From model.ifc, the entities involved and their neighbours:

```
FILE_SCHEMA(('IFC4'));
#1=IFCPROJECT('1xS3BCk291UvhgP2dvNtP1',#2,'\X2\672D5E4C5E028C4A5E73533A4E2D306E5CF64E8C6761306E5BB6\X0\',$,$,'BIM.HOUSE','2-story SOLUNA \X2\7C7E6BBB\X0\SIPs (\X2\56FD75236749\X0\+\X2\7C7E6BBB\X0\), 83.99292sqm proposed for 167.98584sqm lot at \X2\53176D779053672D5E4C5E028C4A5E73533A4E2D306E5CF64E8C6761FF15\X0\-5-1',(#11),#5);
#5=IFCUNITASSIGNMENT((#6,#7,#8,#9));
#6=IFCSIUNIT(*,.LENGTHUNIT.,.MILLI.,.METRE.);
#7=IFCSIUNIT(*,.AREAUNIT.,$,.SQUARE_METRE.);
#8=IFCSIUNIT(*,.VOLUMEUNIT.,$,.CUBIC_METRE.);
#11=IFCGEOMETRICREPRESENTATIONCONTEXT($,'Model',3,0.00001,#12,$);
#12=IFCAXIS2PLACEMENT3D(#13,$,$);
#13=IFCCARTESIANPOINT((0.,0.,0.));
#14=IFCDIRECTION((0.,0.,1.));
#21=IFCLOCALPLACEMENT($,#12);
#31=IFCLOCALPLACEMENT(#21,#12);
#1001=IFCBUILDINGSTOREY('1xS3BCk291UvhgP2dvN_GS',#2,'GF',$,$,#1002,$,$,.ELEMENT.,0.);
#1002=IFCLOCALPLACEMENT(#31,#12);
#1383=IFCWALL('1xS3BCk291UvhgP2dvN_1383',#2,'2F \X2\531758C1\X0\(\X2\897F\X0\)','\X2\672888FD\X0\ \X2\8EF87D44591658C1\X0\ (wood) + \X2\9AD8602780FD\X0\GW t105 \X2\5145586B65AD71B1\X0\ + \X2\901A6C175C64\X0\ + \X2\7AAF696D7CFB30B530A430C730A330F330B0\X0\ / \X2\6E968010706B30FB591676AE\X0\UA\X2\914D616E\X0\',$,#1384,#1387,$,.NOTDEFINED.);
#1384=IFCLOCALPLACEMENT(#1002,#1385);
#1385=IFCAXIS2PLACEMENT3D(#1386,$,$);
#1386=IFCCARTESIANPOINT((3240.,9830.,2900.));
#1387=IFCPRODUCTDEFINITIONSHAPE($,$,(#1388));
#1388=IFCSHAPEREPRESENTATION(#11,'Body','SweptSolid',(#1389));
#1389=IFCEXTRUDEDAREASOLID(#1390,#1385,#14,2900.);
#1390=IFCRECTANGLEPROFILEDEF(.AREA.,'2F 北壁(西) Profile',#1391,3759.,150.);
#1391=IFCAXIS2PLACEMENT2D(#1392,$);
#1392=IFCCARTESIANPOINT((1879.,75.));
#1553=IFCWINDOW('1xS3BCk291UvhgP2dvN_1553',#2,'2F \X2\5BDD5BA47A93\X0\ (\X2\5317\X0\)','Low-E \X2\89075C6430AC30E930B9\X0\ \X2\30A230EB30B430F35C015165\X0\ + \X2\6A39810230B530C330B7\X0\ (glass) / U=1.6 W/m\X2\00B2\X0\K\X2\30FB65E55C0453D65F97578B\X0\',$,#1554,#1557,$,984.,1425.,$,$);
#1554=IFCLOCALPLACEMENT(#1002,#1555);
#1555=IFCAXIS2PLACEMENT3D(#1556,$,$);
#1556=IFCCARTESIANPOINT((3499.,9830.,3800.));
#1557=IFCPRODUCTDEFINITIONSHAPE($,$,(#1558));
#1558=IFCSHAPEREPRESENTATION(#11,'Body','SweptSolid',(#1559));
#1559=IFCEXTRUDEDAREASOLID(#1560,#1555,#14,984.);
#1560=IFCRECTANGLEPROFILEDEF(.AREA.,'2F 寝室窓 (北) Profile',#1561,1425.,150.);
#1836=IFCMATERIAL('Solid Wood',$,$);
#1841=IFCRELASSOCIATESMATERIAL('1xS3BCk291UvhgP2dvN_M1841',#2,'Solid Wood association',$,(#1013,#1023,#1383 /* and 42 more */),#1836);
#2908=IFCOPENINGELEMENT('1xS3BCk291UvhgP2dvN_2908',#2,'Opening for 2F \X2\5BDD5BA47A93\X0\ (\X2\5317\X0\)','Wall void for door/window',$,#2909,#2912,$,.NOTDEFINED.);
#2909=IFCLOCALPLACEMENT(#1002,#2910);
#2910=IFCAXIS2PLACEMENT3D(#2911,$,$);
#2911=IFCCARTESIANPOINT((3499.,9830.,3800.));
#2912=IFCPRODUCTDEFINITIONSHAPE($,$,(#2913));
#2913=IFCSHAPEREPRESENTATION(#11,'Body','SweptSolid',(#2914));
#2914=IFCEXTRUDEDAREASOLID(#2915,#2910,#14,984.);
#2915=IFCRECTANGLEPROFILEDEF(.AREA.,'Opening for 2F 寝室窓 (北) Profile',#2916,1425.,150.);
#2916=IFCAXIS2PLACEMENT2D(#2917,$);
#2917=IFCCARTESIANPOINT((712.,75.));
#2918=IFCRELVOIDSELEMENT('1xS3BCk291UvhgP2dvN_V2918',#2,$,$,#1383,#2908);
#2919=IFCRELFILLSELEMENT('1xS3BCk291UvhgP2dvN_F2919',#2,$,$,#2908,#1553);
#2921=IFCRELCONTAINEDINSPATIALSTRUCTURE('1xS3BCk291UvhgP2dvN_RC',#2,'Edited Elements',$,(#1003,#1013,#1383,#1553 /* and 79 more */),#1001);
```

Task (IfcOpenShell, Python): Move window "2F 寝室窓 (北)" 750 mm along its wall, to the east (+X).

```python
import ifcopenshell
import ifcopenshell.api.geometry
import ifcopenshell.util.placement

model = ifcopenshell.open("model.ifc")

window = model.by_id(1553)
opening = window.FillsVoids[0].RelatingOpeningElement
wall = opening.VoidsElements[0].RelatingBuildingElement

wall_matrix = ifcopenshell.util.placement.get_local_placement(wall.ObjectPlacement)
shift = wall_matrix[:3, 0] * 750.0
before = ifcopenshell.util.placement.get_local_placement(window.ObjectPlacement)[:3, 3].copy()

# The window is not placed relative to its opening, so move both.
for product in (opening, window):
    matrix = ifcopenshell.util.placement.get_local_placement(product.ObjectPlacement)
    matrix[:3, 3] += shift
    ifcopenshell.api.geometry.edit_object_placement(model, product=product, matrix=matrix, is_si=False)

after = ifcopenshell.util.placement.get_local_placement(window.ObjectPlacement)[:3, 3]
print("window moved by", (after - before).round(3) + 0.0)

model.write("model_v2.ifc")
```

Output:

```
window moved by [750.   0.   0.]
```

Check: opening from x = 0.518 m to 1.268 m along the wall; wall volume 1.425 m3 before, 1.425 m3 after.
